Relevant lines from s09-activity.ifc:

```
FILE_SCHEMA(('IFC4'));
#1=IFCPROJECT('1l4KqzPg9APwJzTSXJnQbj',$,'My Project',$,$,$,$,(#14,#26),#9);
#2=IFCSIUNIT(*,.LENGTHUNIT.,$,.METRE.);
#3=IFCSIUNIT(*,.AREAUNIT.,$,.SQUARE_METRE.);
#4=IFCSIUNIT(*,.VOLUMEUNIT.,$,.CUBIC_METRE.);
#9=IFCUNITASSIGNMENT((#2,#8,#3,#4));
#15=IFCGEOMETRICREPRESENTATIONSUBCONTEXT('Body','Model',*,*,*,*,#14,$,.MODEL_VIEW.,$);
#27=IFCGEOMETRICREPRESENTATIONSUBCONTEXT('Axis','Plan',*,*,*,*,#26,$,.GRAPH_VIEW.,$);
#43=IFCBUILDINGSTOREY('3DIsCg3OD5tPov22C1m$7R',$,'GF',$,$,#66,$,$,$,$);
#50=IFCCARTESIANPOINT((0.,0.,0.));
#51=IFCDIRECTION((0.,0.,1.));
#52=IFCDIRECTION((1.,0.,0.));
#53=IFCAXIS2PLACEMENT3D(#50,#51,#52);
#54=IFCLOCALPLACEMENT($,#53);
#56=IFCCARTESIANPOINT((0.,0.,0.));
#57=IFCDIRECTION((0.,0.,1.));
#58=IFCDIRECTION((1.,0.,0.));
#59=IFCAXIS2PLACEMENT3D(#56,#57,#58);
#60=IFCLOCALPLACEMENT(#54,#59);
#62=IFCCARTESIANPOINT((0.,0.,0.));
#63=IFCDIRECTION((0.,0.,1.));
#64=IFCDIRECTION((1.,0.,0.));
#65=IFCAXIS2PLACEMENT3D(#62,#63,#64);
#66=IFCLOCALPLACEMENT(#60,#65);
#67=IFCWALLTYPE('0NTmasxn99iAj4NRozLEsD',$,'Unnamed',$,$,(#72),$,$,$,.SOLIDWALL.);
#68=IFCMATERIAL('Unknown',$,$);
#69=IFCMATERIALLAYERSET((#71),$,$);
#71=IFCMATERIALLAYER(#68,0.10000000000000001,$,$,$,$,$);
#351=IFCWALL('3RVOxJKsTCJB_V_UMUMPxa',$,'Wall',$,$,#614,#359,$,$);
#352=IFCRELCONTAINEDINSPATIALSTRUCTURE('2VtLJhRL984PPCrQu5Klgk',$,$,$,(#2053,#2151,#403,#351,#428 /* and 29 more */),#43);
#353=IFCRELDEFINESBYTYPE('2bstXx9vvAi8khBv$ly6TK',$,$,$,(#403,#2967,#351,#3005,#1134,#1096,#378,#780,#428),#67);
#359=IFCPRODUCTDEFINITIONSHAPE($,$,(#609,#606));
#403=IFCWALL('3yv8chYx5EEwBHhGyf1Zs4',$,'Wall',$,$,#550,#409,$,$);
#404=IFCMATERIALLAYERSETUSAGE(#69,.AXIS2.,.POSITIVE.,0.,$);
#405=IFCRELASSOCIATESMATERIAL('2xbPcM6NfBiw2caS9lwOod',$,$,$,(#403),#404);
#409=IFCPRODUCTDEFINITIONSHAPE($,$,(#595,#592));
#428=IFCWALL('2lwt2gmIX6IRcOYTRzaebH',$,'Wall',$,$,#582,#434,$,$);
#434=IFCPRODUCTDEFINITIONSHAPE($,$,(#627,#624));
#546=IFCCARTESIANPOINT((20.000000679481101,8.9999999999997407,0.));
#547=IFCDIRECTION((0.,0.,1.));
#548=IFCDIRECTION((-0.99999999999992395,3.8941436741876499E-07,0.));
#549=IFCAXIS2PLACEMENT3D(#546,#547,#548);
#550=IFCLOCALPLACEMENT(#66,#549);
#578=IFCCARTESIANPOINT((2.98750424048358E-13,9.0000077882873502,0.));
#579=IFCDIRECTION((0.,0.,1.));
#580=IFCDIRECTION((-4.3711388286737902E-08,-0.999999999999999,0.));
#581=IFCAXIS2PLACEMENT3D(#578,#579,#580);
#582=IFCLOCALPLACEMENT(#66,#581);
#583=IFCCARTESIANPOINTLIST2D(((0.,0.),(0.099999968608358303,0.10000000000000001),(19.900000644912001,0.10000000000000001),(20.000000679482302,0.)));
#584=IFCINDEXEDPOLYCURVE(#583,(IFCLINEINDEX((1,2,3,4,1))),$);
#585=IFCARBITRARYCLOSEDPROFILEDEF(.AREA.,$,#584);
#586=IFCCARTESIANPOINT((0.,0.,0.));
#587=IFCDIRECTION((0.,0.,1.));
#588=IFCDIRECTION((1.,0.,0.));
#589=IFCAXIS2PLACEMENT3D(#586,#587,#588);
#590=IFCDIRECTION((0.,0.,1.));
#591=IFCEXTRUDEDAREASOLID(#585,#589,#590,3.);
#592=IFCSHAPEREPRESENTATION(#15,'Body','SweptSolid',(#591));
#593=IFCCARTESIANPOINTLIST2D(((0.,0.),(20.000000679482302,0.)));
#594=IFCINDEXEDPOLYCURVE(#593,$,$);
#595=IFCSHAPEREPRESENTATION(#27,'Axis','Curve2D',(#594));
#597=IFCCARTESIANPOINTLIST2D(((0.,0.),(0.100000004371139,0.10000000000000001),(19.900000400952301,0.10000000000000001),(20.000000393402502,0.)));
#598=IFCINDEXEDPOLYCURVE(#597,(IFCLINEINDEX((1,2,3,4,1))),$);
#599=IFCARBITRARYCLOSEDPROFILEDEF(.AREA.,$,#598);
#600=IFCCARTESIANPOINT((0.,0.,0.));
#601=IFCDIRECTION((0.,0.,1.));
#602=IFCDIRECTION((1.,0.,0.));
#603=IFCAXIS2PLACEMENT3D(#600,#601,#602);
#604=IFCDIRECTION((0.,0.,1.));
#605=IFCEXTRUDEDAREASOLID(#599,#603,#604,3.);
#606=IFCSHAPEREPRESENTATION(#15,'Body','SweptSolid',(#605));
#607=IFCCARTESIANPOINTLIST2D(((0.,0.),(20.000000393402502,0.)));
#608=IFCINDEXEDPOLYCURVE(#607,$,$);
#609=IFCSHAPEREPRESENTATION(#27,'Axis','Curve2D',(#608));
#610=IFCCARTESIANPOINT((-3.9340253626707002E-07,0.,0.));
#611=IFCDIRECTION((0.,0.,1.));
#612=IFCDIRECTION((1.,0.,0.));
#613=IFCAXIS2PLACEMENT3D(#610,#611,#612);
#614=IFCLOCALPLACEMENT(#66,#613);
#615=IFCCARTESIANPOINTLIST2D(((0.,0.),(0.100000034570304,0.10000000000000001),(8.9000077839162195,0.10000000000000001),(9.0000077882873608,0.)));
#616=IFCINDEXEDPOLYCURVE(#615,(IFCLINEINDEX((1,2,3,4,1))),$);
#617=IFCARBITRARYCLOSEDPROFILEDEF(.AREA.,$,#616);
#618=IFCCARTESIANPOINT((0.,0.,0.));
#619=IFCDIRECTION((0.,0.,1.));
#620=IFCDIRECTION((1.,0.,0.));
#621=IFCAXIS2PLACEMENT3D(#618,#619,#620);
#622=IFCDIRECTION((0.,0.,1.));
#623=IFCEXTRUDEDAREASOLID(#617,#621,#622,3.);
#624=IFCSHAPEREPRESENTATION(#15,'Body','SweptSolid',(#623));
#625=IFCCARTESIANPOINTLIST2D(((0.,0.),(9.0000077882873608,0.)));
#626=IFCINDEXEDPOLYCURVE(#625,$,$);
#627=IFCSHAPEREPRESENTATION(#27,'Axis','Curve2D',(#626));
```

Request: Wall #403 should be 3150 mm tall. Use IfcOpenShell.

```python
import ifcopenshell
import ifcopenshell.geom
import ifcopenshell.util.representation
import ifcopenshell.util.shape
import ifcopenshell.util.unit

model = ifcopenshell.open("s09-activity.ifc")
unit_scale = ifcopenshell.util.unit.calculate_unit_scale(model)
settings = ifcopenshell.geom.settings()


def volume(element):
    """Net volume in cubic metres, openings subtracted."""
    shape = ifcopenshell.geom.create_shape(settings, element)
    return ifcopenshell.util.shape.get_volume(shape.geometry)


wall = model.by_guid("3yv8chYx5EEwBHhGyf1Zs4")
before = volume(wall)

body = ifcopenshell.util.representation.get_representation(wall, "Model", "Body")
solid = body.Items[0]
old_height = solid.Depth
solid.Depth = 3.15 / unit_scale
after = volume(wall)

print(f"height {old_height:g} -> {solid.Depth:g}, volume {before:.3f} -> {after:.3f} m3")

model.write("s09-activity_edited.ifc")
```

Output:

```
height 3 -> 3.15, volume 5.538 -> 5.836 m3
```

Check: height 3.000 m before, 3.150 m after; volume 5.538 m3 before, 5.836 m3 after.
